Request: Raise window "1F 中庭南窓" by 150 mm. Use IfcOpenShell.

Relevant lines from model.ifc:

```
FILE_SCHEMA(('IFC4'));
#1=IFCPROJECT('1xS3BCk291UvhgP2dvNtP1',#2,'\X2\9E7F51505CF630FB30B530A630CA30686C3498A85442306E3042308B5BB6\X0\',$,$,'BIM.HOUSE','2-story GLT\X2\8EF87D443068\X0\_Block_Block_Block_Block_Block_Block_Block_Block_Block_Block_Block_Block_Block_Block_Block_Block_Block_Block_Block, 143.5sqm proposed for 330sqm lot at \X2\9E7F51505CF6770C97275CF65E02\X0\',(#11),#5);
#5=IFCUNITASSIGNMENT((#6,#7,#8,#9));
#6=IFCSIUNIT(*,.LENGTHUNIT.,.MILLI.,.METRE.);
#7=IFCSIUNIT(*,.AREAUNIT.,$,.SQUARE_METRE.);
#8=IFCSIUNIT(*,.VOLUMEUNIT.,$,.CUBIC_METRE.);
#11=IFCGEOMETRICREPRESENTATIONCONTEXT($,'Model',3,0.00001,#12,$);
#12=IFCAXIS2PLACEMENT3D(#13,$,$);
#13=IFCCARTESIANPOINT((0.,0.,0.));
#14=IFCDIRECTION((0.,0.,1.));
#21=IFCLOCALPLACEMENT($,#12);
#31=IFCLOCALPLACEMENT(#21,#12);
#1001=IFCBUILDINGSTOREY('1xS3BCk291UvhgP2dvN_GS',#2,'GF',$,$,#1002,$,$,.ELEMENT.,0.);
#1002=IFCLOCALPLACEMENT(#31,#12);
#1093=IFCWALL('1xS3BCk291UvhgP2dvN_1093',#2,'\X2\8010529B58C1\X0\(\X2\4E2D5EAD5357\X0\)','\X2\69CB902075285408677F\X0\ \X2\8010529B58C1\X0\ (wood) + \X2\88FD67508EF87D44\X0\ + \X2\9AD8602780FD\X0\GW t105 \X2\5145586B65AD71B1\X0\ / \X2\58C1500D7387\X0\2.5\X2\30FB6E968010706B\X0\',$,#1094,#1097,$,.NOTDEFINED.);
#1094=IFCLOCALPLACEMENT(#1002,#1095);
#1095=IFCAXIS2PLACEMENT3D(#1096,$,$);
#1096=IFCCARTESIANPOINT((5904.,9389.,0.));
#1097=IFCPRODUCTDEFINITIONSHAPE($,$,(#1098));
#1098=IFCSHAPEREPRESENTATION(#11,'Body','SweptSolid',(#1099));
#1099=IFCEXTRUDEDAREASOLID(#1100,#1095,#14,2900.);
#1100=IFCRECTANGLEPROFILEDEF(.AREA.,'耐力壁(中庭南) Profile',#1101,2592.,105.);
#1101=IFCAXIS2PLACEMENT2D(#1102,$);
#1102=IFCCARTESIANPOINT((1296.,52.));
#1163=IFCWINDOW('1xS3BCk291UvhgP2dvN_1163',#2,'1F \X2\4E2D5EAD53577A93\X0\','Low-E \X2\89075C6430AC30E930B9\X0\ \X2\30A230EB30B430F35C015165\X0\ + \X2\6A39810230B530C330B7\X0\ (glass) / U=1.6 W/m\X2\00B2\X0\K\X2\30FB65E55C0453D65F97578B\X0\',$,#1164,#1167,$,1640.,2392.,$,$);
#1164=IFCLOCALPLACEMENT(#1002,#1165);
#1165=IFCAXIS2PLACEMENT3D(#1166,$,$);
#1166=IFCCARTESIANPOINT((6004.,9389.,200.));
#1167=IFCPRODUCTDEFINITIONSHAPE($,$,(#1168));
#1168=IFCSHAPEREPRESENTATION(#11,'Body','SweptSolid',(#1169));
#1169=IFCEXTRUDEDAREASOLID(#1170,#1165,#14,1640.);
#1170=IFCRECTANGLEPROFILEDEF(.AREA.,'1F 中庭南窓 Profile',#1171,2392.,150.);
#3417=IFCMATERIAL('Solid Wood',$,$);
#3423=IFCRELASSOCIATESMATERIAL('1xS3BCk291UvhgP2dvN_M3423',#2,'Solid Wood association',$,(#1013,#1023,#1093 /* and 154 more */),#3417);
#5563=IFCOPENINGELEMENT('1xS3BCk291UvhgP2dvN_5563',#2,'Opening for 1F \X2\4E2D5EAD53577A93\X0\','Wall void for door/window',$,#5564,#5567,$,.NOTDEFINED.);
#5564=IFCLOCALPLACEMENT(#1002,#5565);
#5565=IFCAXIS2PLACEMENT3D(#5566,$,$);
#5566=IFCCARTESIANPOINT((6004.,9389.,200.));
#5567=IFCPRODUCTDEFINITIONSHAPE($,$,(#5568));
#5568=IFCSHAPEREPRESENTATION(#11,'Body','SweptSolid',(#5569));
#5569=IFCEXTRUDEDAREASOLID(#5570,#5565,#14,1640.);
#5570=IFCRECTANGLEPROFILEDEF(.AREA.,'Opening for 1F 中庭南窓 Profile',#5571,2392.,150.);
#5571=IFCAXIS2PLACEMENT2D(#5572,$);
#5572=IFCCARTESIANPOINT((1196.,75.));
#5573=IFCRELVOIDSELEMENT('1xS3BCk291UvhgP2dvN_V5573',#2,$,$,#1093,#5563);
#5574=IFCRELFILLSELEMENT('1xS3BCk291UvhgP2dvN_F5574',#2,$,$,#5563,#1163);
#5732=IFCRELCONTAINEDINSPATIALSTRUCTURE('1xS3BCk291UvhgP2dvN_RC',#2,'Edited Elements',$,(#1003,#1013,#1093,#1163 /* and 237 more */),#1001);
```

```python
import numpy as np
import ifcopenshell
import ifcopenshell.api.geometry
import ifcopenshell.util.placement
import ifcopenshell.util.unit

model = ifcopenshell.open("model.ifc")
unit_scale = ifcopenshell.util.unit.calculate_unit_scale(model)

window = model.by_guid("1xS3BCk291UvhgP2dvN_1163")
opening = window.FillsVoids[0].RelatingOpeningElement
dz = 150.0

shift = np.array([0.0, 0.0, dz])
# The window is not placed relative to its opening, so move both.
for product in (opening, window):
    matrix = ifcopenshell.util.placement.get_local_placement(product.ObjectPlacement)
    matrix[:3, 3] += shift
    ifcopenshell.api.geometry.edit_object_placement(model, product=product, matrix=matrix, is_si=False)

print(f"moved by {dz * unit_scale:+.3f} m")

model.write("model_rev.ifc")
```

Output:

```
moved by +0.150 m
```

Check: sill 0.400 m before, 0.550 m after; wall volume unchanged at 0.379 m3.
